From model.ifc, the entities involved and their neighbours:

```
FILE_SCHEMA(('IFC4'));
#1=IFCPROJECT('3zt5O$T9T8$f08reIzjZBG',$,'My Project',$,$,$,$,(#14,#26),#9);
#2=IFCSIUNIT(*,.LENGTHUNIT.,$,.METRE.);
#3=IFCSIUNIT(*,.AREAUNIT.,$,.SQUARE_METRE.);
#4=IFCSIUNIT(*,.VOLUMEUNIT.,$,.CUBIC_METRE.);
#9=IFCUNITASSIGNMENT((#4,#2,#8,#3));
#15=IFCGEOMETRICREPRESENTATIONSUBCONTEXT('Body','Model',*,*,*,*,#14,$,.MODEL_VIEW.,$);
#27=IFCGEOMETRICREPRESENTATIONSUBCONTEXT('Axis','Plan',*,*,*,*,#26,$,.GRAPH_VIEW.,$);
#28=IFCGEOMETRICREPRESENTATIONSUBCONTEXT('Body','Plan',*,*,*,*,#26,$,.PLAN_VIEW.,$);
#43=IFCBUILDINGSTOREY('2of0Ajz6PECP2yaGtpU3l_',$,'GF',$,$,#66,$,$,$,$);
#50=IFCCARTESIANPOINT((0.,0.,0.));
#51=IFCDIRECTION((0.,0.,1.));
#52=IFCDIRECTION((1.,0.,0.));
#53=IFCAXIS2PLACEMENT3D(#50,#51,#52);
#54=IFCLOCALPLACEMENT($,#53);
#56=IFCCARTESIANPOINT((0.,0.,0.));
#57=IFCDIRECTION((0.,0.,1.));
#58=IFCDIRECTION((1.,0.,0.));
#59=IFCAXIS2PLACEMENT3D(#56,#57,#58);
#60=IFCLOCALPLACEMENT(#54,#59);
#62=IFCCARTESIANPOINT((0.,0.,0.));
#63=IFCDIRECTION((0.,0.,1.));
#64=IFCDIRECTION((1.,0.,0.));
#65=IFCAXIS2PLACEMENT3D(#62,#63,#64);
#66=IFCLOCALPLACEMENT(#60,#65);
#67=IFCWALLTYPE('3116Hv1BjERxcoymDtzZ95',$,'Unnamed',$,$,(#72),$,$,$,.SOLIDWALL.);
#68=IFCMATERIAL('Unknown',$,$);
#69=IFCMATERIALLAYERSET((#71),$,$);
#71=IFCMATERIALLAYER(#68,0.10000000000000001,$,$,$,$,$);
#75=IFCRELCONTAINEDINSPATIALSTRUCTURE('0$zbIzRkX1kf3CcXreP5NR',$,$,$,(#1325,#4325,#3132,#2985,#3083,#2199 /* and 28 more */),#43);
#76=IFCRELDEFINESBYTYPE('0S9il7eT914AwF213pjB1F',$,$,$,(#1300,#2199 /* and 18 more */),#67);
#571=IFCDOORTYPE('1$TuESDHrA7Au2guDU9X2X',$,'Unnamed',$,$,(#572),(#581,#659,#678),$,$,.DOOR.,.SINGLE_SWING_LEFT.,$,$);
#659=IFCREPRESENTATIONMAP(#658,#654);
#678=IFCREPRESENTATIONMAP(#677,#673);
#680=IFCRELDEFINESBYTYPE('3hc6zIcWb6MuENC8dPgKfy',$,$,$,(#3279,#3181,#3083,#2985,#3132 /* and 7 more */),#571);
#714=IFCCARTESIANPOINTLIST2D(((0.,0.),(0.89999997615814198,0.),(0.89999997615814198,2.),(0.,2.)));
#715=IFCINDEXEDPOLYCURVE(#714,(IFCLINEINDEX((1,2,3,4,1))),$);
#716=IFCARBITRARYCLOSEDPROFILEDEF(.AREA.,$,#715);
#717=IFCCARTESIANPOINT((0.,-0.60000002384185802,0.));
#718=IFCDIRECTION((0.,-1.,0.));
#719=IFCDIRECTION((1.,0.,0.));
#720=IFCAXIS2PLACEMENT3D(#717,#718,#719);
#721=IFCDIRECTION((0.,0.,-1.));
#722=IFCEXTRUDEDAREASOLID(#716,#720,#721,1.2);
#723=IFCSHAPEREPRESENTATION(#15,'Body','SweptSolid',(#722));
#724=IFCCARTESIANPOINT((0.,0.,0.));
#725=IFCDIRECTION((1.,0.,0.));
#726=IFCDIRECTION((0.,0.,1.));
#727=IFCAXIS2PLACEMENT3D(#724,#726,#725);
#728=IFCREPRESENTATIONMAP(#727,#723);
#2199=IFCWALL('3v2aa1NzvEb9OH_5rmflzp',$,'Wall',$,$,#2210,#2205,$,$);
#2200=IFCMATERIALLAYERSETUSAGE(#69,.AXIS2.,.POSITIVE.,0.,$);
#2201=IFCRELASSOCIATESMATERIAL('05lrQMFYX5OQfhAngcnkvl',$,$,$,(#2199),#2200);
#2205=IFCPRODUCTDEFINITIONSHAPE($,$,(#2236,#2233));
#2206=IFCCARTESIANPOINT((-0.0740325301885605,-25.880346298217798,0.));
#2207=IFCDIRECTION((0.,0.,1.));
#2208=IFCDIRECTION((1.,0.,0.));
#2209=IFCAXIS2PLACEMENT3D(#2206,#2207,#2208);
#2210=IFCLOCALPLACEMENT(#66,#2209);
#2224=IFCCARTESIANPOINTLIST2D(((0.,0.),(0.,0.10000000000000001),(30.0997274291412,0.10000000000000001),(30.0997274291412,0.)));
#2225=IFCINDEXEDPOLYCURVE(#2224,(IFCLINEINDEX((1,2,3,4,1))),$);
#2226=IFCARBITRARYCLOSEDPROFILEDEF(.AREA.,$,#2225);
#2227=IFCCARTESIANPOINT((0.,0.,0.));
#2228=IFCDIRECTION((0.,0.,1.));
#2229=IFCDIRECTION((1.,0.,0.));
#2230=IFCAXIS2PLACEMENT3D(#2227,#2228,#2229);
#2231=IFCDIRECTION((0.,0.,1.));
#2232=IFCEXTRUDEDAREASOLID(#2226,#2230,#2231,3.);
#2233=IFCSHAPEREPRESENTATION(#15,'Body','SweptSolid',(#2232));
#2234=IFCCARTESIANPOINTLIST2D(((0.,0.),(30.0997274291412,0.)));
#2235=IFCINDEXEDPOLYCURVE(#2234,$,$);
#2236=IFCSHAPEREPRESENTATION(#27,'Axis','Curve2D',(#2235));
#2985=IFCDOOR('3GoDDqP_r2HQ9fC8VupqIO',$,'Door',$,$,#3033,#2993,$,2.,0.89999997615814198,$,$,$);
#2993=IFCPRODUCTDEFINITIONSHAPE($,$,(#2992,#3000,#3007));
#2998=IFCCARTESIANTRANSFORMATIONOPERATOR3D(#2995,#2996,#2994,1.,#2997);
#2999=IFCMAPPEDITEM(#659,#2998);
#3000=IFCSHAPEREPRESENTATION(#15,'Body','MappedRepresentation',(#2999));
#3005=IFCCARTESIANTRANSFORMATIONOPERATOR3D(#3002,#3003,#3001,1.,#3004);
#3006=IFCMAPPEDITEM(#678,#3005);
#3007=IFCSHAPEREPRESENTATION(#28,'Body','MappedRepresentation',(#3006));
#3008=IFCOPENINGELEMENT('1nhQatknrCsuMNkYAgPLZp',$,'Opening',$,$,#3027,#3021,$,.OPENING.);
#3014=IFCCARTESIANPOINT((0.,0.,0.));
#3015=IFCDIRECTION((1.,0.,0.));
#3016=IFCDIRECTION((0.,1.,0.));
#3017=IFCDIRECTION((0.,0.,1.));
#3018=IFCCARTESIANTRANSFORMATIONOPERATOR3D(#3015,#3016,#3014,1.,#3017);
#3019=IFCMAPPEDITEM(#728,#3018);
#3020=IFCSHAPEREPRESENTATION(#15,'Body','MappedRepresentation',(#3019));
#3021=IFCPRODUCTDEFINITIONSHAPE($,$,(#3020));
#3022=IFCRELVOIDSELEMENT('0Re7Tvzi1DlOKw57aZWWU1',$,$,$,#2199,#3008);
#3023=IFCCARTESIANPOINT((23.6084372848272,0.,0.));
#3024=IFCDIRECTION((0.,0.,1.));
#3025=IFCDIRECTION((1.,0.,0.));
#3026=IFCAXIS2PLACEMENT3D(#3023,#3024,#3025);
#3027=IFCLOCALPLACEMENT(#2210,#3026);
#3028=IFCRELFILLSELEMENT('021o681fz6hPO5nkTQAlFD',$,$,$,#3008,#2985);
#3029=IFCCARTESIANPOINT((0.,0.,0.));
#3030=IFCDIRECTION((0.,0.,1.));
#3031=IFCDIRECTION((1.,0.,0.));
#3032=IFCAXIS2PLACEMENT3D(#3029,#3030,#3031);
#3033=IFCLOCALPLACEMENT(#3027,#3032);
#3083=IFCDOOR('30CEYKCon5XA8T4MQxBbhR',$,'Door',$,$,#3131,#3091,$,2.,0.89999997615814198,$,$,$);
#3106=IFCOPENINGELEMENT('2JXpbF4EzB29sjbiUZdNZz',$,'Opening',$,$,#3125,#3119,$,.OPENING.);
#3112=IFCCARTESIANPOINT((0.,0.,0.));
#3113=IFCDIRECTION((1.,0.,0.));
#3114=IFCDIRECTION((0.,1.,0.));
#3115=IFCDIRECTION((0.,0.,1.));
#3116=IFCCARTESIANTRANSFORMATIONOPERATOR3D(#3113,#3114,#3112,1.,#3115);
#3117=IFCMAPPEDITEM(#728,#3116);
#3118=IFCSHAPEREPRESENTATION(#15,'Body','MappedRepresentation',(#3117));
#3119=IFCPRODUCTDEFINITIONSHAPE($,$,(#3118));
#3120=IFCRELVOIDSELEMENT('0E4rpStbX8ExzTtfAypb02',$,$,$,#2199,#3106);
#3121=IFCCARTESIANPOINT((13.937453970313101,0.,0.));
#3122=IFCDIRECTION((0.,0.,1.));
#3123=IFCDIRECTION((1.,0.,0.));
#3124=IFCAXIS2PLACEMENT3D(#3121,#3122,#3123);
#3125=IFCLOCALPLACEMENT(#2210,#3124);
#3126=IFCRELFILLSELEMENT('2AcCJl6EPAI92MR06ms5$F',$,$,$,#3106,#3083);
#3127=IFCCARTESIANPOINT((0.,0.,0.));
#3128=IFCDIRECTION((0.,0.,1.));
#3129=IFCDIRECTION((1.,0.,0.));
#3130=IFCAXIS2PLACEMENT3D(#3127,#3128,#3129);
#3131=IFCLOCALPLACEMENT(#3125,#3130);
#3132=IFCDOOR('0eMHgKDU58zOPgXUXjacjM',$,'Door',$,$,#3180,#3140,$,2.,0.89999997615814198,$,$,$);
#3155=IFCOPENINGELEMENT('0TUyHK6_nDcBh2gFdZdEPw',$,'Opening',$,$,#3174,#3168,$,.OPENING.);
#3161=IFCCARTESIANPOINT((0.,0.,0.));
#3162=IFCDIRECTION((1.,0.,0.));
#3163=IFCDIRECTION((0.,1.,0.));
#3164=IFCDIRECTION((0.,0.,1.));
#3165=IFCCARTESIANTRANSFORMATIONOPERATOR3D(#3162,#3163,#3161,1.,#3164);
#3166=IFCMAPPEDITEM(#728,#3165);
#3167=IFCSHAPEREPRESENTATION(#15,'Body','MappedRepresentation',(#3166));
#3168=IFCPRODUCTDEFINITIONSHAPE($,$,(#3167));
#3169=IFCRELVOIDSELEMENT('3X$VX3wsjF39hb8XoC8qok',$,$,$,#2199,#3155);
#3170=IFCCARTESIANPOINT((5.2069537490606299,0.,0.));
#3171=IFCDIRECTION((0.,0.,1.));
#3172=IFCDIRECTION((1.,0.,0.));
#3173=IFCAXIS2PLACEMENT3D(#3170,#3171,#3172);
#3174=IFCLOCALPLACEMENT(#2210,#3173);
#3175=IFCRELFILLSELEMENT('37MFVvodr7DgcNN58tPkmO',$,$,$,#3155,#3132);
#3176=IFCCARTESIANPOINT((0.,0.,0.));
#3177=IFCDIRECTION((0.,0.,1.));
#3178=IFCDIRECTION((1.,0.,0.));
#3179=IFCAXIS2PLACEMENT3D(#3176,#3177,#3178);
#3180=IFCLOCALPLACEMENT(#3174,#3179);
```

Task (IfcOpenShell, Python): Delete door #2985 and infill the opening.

```python
import ifcopenshell
import ifcopenshell.api.feature
import ifcopenshell.api.root
import ifcopenshell.geom
import ifcopenshell.util.shape

model = ifcopenshell.open("model.ifc")
settings = ifcopenshell.geom.settings()


def volume(element):
    """Net volume in cubic metres, openings subtracted."""
    shape = ifcopenshell.geom.create_shape(settings, element)
    return ifcopenshell.util.shape.get_volume(shape.geometry)


door = model.by_guid("3GoDDqP_r2HQ9fC8VupqIO")
opening = door.FillsVoids[0].RelatingOpeningElement
wall = opening.VoidsElements[0].RelatingBuildingElement
before = volume(wall)

ifcopenshell.api.root.remove_product(model, product=door)
ifcopenshell.api.feature.remove_feature(model, feature=opening)

after = volume(wall)

print(f"wall volume {before:.3f} -> {after:.3f} m3")

model.write("model_edited.ifc")
```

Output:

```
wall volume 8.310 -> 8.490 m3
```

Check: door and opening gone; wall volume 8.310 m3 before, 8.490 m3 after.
